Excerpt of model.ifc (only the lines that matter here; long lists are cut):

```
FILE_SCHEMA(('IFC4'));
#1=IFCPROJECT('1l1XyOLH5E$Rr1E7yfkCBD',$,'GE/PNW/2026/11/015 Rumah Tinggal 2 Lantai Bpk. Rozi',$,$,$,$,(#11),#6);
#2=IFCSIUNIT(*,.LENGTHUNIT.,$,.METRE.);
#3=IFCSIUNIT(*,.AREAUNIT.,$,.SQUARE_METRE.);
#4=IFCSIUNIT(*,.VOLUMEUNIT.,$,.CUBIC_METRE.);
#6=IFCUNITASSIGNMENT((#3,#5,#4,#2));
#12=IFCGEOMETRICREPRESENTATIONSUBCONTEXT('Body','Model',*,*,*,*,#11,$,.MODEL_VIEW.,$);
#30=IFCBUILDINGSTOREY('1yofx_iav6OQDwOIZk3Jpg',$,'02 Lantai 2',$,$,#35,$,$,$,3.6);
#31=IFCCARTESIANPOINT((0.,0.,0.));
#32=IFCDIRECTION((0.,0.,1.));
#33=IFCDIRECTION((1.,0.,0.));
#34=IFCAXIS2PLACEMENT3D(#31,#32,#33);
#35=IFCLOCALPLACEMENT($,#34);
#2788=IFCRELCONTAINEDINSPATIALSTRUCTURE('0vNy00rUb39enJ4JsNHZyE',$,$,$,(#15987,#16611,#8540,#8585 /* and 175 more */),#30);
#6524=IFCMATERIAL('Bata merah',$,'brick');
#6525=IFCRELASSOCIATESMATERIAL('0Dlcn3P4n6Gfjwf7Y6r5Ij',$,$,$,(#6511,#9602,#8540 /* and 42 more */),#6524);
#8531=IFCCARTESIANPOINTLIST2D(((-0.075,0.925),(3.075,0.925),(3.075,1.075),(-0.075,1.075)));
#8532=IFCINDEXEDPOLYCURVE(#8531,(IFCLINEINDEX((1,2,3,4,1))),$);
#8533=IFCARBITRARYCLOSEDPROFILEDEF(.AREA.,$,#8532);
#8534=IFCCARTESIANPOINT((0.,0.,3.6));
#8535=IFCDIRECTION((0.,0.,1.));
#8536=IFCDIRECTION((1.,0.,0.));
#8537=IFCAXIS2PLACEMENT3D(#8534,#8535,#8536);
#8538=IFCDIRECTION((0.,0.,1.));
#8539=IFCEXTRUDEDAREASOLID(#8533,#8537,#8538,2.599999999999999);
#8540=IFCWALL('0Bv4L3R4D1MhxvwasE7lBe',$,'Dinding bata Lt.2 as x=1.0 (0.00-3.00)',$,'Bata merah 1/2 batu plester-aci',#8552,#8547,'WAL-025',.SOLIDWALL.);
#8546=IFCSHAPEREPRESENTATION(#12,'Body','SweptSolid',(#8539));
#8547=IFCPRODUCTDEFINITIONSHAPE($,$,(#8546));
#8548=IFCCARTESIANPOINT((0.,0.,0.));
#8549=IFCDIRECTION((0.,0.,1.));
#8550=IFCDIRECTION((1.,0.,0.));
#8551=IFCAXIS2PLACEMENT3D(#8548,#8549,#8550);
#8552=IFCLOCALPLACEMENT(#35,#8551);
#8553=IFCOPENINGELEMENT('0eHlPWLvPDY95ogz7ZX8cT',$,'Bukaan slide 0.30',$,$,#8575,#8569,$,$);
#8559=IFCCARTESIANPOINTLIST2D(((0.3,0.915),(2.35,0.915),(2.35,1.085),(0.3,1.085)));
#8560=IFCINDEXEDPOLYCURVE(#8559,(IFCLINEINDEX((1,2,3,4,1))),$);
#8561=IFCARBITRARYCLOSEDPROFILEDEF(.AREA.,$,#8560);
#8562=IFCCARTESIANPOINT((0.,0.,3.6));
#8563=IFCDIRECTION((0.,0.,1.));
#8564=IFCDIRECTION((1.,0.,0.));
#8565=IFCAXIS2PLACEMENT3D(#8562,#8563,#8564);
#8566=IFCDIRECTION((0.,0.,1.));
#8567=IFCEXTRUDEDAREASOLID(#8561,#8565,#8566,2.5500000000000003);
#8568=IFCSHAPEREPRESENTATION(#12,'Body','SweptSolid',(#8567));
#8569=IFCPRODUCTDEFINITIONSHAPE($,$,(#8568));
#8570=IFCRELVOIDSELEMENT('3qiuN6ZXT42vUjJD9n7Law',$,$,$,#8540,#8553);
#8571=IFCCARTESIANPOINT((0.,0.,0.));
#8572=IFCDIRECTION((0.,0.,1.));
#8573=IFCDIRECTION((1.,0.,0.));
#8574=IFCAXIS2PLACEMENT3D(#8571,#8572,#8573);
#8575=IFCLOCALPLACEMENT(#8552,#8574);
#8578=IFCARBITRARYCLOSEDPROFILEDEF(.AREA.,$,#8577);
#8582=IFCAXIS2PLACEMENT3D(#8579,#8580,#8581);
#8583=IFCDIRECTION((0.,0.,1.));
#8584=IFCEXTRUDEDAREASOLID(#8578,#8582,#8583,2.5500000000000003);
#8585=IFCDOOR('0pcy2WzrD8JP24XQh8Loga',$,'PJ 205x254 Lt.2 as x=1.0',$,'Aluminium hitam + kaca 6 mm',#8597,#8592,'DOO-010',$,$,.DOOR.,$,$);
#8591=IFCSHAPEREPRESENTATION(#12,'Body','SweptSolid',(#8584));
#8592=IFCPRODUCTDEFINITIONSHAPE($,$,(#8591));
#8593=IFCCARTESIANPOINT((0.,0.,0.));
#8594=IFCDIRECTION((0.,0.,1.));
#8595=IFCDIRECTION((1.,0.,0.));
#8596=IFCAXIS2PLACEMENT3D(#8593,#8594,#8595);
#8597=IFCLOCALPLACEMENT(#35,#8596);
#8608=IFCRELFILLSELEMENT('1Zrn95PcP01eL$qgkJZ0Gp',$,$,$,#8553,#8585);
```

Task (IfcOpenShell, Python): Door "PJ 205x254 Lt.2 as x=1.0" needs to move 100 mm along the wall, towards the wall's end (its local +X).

```python
import ifcopenshell
import ifcopenshell.api.geometry
import ifcopenshell.util.placement

model = ifcopenshell.open("model.ifc")

door = model.by_guid("0pcy2WzrD8JP24XQh8Loga")
opening = door.FillsVoids[0].RelatingOpeningElement
wall = opening.VoidsElements[0].RelatingBuildingElement

wall_matrix = ifcopenshell.util.placement.get_local_placement(wall.ObjectPlacement)
shift = wall_matrix[:3, 0] * 0.1
before = ifcopenshell.util.placement.get_local_placement(door.ObjectPlacement)[:3, 3].copy()

# The door is not placed relative to its opening, so move both.
for product in (opening, door):
    matrix = ifcopenshell.util.placement.get_local_placement(product.ObjectPlacement)
    matrix[:3, 3] += shift
    ifcopenshell.api.geometry.edit_object_placement(model, product=product, matrix=matrix, is_si=False)

after = ifcopenshell.util.placement.get_local_placement(door.ObjectPlacement)[:3, 3]
print("door moved by", (after - before).round(3) + 0.0)

model.write("model-out.ifc")
```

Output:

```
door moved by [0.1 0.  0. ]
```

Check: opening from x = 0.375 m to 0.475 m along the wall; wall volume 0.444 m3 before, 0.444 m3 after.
